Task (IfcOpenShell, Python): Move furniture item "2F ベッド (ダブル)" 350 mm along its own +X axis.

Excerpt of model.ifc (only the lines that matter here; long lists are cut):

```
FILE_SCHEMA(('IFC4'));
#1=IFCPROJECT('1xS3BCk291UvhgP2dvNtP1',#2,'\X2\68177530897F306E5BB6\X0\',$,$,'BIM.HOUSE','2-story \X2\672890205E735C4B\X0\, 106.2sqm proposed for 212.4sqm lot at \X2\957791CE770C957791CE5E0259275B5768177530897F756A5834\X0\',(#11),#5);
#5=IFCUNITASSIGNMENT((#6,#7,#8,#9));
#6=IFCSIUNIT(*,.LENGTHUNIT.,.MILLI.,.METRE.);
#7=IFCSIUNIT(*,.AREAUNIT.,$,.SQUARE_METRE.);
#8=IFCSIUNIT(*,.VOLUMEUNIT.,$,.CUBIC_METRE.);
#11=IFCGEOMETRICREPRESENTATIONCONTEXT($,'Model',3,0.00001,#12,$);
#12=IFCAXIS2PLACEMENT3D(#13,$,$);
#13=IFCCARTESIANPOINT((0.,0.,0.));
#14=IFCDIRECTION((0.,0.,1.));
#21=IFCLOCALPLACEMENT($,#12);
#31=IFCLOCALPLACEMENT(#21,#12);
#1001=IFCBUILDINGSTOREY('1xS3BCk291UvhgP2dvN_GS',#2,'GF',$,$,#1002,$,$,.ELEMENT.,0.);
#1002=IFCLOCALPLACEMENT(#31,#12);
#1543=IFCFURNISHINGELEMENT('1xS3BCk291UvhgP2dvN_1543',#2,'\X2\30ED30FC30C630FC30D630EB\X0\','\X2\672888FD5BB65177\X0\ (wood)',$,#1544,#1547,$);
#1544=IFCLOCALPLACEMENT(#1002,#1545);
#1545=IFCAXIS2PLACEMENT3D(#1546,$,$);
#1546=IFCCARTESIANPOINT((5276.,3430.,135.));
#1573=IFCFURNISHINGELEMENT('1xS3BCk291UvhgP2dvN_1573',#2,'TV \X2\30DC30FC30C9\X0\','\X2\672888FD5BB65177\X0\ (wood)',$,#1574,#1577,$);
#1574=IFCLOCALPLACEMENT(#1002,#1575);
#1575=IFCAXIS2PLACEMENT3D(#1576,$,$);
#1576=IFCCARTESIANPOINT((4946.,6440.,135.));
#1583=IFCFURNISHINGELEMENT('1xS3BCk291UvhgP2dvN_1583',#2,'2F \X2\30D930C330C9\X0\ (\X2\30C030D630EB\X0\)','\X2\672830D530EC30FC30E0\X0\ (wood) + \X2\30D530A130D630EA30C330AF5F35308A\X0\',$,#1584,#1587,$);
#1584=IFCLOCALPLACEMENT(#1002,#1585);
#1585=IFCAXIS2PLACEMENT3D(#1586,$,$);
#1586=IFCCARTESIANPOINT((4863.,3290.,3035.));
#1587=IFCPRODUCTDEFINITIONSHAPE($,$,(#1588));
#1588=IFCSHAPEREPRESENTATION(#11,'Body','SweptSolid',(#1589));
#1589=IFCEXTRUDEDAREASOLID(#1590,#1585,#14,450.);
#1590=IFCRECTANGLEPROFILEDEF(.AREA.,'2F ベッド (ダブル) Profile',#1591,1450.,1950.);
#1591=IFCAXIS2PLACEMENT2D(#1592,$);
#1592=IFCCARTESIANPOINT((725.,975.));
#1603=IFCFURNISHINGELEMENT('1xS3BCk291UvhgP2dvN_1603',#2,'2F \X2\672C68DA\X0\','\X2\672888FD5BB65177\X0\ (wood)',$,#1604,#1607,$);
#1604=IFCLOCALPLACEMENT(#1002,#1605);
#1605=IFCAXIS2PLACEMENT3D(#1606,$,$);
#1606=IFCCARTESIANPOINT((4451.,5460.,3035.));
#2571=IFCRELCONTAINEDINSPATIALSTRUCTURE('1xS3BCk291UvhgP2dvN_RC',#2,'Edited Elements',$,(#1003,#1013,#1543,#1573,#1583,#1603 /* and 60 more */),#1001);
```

```python
import ifcopenshell
import ifcopenshell.api.geometry
import ifcopenshell.util.placement
import ifcopenshell.util.unit

model = ifcopenshell.open("model.ifc")
unit_scale = ifcopenshell.util.unit.calculate_unit_scale(model)

item = model.by_id(1583)
matrix = ifcopenshell.util.placement.get_local_placement(item.ObjectPlacement)
matrix[:3, 3] += matrix[:3, 0] * 0.35 / unit_scale
ifcopenshell.api.geometry.edit_object_placement(model, product=item, matrix=matrix, is_si=False)

print(ifcopenshell.util.placement.get_local_placement(item.ObjectPlacement).round(3) + 0.0)

model.write("model_edited.ifc")
```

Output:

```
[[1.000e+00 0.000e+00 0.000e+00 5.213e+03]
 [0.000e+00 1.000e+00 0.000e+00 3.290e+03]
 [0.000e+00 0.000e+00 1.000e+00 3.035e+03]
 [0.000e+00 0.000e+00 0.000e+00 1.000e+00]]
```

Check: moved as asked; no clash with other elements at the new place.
